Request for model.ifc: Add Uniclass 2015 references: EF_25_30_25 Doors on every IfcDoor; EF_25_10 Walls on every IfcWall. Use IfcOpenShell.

First a look at what the model holds.

```python
import ifcopenshell

model = ifcopenshell.open("model.ifc")
print(model.schema)
print("classifications:", [c.Name for c in model.by_type("IfcClassification")])
for ifc_class in ("IfcDoor", "IfcRoof", "IfcStair", "IfcWall", "IfcWindow"):
    print(ifc_class, len(model.by_type(ifc_class)))
```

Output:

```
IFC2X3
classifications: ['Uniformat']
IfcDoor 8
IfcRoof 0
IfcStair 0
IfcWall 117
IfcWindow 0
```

```python
import ifcopenshell
import ifcopenshell.api.classification

model = ifcopenshell.open("model.ifc")

# IFC2X3 requires Source and Edition and has no link from the project to the system.
system = model.create_entity("IfcClassification", Source="NBS", Edition="2015", Name="Uniclass 2015")

codes = {
    "IfcDoor": ("EF_25_30_25", "Doors"),
    "IfcWall": ("EF_25_10", "Walls"),
}
for ifc_class, (code, name) in codes.items():
    products = model.by_type(ifc_class)
    ifcopenshell.api.classification.add_reference(
        model, products=products, classification=system, identification=code, name=name
    )
    print(code, len(products))

model.write("model_updated.ifc")
```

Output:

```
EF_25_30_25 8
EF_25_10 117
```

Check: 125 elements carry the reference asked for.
